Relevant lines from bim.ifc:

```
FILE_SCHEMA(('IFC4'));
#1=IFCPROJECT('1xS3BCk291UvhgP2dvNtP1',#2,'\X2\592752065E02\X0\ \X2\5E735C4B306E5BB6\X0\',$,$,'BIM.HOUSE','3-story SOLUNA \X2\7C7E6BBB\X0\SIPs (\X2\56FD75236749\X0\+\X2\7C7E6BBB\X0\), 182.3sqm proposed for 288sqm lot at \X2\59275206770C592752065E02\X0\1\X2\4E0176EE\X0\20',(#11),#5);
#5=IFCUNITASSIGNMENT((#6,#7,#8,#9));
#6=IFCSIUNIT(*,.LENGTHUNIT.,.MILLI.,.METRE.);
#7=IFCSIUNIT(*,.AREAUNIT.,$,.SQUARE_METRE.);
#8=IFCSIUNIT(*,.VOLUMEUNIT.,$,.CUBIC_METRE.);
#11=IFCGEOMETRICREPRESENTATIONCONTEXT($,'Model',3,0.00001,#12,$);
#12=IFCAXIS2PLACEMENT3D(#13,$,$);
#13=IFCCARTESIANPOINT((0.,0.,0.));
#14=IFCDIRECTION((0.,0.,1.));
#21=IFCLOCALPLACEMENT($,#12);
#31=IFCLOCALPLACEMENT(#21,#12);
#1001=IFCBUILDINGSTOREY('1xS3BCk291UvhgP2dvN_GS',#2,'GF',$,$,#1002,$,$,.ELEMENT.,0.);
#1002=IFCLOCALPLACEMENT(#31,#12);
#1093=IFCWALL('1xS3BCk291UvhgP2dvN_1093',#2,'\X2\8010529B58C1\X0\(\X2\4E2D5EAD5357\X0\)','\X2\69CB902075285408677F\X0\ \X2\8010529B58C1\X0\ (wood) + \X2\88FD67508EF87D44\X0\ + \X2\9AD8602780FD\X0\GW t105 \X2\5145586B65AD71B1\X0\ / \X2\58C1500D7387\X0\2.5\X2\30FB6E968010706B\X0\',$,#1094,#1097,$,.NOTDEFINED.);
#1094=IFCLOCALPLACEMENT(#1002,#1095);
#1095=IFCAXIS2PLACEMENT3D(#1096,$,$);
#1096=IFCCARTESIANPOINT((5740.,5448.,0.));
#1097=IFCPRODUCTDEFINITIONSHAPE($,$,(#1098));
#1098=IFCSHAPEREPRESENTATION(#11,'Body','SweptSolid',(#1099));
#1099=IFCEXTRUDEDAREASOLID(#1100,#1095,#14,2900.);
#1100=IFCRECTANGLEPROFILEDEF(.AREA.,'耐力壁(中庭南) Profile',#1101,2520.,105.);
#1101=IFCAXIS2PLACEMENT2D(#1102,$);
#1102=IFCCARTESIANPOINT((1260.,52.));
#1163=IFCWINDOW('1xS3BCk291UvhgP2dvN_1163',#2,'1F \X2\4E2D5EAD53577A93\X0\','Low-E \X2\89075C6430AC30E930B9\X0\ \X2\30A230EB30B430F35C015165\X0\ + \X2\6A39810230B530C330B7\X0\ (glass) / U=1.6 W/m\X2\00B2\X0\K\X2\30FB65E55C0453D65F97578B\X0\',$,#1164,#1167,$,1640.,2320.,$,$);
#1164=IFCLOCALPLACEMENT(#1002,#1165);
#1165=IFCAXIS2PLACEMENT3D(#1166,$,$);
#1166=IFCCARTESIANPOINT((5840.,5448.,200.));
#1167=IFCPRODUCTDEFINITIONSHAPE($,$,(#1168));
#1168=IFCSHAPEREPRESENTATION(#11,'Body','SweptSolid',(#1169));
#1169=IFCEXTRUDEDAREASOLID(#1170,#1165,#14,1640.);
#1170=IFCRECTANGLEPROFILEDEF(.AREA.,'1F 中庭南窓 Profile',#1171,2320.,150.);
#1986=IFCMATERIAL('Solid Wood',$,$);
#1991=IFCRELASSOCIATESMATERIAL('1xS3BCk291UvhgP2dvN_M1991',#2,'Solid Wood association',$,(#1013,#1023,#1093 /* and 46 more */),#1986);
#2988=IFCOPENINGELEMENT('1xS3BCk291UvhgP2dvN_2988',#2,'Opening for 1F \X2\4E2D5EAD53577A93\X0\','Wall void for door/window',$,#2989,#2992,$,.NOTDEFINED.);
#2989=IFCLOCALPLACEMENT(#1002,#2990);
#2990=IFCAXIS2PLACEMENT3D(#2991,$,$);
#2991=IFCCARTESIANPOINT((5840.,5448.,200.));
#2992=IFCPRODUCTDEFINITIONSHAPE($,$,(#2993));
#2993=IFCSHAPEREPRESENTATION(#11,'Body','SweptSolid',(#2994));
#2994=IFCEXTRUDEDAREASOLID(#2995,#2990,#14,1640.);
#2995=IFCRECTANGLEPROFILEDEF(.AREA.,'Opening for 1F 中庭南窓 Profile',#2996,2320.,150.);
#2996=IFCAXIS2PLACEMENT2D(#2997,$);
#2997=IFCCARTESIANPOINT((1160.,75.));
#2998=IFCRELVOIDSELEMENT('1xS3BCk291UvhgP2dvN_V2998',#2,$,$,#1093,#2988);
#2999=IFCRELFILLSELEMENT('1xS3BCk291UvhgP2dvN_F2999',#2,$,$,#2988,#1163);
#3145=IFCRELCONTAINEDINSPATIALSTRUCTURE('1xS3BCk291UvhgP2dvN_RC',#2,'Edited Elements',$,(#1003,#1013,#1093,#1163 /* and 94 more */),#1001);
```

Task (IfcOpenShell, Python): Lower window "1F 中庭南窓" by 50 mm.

```python
import numpy as np
import ifcopenshell
import ifcopenshell.api.geometry
import ifcopenshell.util.placement
import ifcopenshell.util.unit

model = ifcopenshell.open("bim.ifc")
unit_scale = ifcopenshell.util.unit.calculate_unit_scale(model)

window = model.by_guid("1xS3BCk291UvhgP2dvN_1163")
opening = window.FillsVoids[0].RelatingOpeningElement
dz = -0.05 / unit_scale

shift = np.array([0.0, 0.0, dz])
# The window is not placed relative to its opening, so move both.
for product in (opening, window):
    matrix = ifcopenshell.util.placement.get_local_placement(product.ObjectPlacement)
    matrix[:3, 3] += shift
    ifcopenshell.api.geometry.edit_object_placement(model, product=product, matrix=matrix, is_si=False)

print(f"moved by {dz * unit_scale:+.3f} m")

model.write("bim-out.ifc")
```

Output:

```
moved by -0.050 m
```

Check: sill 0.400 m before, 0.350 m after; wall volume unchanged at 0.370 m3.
